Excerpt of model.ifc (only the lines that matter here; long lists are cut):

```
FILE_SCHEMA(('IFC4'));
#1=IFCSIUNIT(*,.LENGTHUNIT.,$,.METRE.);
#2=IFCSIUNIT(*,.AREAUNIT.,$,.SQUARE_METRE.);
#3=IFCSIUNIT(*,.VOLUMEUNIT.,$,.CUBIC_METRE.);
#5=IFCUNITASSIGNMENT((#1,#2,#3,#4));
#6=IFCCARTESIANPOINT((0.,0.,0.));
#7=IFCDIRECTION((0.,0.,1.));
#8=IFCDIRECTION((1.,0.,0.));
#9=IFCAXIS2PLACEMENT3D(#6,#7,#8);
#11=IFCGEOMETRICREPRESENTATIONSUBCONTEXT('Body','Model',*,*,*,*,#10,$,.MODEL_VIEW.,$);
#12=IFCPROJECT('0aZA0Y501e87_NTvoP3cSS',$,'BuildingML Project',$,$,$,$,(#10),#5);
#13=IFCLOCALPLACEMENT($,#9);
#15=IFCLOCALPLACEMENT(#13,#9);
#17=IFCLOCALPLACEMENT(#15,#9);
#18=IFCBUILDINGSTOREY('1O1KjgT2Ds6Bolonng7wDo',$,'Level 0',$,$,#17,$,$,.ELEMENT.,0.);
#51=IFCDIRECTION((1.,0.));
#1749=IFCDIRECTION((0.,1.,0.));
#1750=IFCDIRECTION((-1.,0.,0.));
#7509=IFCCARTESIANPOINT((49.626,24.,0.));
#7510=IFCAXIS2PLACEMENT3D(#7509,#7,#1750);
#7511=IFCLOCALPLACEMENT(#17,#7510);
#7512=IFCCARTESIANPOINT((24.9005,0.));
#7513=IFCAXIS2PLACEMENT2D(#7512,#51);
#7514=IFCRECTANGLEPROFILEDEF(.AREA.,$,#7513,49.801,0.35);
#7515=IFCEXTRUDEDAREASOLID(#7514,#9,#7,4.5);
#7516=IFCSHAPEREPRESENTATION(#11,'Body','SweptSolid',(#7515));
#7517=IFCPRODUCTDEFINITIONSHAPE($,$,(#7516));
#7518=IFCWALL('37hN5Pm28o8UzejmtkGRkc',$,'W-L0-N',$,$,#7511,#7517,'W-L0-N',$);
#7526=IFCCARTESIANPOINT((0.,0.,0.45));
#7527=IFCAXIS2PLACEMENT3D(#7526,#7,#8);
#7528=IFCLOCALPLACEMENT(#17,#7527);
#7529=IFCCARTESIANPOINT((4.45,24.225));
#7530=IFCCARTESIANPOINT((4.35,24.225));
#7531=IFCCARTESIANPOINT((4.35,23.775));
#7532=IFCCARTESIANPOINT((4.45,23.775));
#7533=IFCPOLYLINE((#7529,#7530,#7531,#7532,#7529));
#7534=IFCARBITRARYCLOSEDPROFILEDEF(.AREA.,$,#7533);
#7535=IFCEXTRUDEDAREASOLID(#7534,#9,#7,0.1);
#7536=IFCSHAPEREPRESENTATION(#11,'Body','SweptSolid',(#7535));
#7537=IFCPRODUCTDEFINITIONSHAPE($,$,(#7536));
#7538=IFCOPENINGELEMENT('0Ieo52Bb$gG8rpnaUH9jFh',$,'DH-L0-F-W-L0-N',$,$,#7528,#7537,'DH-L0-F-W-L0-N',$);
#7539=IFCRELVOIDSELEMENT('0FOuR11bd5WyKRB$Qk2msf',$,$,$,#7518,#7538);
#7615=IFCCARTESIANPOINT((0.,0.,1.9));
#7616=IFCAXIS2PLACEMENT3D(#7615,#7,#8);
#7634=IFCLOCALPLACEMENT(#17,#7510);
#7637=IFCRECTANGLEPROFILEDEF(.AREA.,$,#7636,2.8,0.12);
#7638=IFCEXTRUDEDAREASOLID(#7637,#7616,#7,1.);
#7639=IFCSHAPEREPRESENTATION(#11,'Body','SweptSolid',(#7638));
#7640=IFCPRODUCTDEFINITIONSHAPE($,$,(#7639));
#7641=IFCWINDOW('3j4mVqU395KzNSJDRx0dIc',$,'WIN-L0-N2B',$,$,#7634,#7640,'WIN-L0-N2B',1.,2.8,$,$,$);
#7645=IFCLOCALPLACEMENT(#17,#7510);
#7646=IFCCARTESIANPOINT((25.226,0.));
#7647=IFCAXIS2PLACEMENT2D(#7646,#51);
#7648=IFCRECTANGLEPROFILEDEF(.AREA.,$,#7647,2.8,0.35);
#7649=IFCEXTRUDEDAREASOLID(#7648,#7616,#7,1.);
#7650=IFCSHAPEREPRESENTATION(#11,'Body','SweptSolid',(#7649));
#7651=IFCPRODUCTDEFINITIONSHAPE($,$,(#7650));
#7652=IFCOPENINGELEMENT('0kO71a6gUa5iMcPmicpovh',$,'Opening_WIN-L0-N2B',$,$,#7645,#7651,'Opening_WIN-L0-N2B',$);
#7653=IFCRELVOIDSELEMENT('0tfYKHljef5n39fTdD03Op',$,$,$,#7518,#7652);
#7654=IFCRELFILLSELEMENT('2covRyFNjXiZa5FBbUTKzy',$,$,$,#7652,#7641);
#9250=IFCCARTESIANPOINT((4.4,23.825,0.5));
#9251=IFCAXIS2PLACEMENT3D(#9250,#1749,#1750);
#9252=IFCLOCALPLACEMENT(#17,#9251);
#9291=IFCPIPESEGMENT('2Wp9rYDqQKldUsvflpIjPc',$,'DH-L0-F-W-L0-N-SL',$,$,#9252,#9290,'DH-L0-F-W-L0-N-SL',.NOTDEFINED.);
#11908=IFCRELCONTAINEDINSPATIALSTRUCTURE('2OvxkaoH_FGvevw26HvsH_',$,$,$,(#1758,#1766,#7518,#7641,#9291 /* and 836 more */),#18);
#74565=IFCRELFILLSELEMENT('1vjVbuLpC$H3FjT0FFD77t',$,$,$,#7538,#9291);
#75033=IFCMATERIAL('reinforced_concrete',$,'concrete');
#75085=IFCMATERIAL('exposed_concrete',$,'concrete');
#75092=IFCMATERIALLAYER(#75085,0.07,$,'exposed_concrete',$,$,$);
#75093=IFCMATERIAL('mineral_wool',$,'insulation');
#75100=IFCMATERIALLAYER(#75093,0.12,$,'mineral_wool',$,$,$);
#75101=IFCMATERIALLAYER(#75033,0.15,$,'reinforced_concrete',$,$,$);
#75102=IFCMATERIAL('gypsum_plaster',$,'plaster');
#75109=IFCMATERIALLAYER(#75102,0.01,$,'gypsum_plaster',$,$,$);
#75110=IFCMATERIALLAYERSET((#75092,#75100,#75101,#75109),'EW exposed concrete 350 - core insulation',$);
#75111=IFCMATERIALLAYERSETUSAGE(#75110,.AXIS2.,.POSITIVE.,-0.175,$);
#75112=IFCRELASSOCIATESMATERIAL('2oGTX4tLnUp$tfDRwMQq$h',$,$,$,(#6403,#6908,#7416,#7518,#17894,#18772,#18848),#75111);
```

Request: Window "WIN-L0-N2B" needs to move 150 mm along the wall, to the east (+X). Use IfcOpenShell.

```python
import ifcopenshell
import ifcopenshell.api.geometry
import ifcopenshell.util.placement
import ifcopenshell.util.unit

model = ifcopenshell.open("model.ifc")
unit_scale = ifcopenshell.util.unit.calculate_unit_scale(model)

window = model.by_guid("3j4mVqU395KzNSJDRx0dIc")
opening = window.FillsVoids[0].RelatingOpeningElement
wall = opening.VoidsElements[0].RelatingBuildingElement

wall_matrix = ifcopenshell.util.placement.get_local_placement(wall.ObjectPlacement)
shift = wall_matrix[:3, 0] * -0.15 / unit_scale
before = ifcopenshell.util.placement.get_local_placement(window.ObjectPlacement)[:3, 3].copy()

# The window is not placed relative to its opening, so move both.
for product in (opening, window):
    matrix = ifcopenshell.util.placement.get_local_placement(product.ObjectPlacement)
    matrix[:3, 3] += shift
    ifcopenshell.api.geometry.edit_object_placement(model, product=product, matrix=matrix, is_si=False)

after = ifcopenshell.util.placement.get_local_placement(window.ObjectPlacement)[:3, 3]
print("window moved by", (after - before).round(3) + 0.0)

model.write("model-out.ifc")
```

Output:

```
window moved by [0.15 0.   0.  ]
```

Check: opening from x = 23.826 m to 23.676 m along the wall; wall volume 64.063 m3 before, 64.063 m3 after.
